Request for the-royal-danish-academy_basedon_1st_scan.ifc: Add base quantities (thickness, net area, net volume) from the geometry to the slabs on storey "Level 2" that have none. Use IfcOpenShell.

First a look at what the model holds.

```python
import ifcopenshell
import ifcopenshell.util.element
import ifcopenshell.util.unit

model = ifcopenshell.open("the-royal-danish-academy_basedon_1st_scan.ifc")
print(model.schema)
for unit_type in ("LENGTHUNIT", "AREAUNIT", "VOLUMEUNIT"):
    print(unit_type, ifcopenshell.util.unit.calculate_unit_scale(model, unit_type))
storey = next(s for s in model.by_type("IfcBuildingStorey") if s.Name == "Level 2")
slabs = [e for e in ifcopenshell.util.element.get_decomposition(storey) if e.is_a("IfcSlab")]
for e in sorted(slabs, key=lambda e: e.id()):
    print(e.id(), e.is_a(), e.Name, list(ifcopenshell.util.element.get_psets(e, qtos_only=True)), sep=" | ")
```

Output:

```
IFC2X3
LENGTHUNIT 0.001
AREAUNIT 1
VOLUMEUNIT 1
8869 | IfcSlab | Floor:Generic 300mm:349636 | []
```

```python
import ifcopenshell
import ifcopenshell.api.pset
import ifcopenshell.geom
import ifcopenshell.util.element
import ifcopenshell.util.shape
import ifcopenshell.util.unit

model = ifcopenshell.open("the-royal-danish-academy_basedon_1st_scan.ifc")
unit_scale = ifcopenshell.util.unit.calculate_unit_scale(model)
area_scale = ifcopenshell.util.unit.calculate_unit_scale(model, "AREAUNIT")
volume_scale = ifcopenshell.util.unit.calculate_unit_scale(model, "VOLUMEUNIT")
settings = ifcopenshell.geom.settings()

storey = next(s for s in model.by_type("IfcBuildingStorey") if s.Name == "Level 2")
slabs = [e for e in ifcopenshell.util.element.get_decomposition(storey) if e.is_a("IfcSlab")]

for e in sorted(slabs, key=lambda e: e.id()):
    if ifcopenshell.util.element.get_psets(e, qtos_only=True, should_inherit=False):
        continue
    # Geometry comes back in metres, in the element's own axes.
    shape = ifcopenshell.geom.create_shape(settings, e)
    values = {
        "Width": ifcopenshell.util.shape.get_z(shape.geometry) / unit_scale,
        "NetArea": ifcopenshell.util.shape.get_footprint_area(shape.geometry) / area_scale,
        "NetVolume": ifcopenshell.util.shape.get_volume(shape.geometry) / volume_scale,
    }
    qto = ifcopenshell.api.pset.add_qto(model, product=e, name="BaseQuantities")
    ifcopenshell.api.pset.edit_qto(model, qto=qto, properties=values)
    print(e.id(), {k: round(v, 3) for k, v in values.items()})

model.write("the-royal-danish-academy_basedon_1st_scan_rev.ifc")
```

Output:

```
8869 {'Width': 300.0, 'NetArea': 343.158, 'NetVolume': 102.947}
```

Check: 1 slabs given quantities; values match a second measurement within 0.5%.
